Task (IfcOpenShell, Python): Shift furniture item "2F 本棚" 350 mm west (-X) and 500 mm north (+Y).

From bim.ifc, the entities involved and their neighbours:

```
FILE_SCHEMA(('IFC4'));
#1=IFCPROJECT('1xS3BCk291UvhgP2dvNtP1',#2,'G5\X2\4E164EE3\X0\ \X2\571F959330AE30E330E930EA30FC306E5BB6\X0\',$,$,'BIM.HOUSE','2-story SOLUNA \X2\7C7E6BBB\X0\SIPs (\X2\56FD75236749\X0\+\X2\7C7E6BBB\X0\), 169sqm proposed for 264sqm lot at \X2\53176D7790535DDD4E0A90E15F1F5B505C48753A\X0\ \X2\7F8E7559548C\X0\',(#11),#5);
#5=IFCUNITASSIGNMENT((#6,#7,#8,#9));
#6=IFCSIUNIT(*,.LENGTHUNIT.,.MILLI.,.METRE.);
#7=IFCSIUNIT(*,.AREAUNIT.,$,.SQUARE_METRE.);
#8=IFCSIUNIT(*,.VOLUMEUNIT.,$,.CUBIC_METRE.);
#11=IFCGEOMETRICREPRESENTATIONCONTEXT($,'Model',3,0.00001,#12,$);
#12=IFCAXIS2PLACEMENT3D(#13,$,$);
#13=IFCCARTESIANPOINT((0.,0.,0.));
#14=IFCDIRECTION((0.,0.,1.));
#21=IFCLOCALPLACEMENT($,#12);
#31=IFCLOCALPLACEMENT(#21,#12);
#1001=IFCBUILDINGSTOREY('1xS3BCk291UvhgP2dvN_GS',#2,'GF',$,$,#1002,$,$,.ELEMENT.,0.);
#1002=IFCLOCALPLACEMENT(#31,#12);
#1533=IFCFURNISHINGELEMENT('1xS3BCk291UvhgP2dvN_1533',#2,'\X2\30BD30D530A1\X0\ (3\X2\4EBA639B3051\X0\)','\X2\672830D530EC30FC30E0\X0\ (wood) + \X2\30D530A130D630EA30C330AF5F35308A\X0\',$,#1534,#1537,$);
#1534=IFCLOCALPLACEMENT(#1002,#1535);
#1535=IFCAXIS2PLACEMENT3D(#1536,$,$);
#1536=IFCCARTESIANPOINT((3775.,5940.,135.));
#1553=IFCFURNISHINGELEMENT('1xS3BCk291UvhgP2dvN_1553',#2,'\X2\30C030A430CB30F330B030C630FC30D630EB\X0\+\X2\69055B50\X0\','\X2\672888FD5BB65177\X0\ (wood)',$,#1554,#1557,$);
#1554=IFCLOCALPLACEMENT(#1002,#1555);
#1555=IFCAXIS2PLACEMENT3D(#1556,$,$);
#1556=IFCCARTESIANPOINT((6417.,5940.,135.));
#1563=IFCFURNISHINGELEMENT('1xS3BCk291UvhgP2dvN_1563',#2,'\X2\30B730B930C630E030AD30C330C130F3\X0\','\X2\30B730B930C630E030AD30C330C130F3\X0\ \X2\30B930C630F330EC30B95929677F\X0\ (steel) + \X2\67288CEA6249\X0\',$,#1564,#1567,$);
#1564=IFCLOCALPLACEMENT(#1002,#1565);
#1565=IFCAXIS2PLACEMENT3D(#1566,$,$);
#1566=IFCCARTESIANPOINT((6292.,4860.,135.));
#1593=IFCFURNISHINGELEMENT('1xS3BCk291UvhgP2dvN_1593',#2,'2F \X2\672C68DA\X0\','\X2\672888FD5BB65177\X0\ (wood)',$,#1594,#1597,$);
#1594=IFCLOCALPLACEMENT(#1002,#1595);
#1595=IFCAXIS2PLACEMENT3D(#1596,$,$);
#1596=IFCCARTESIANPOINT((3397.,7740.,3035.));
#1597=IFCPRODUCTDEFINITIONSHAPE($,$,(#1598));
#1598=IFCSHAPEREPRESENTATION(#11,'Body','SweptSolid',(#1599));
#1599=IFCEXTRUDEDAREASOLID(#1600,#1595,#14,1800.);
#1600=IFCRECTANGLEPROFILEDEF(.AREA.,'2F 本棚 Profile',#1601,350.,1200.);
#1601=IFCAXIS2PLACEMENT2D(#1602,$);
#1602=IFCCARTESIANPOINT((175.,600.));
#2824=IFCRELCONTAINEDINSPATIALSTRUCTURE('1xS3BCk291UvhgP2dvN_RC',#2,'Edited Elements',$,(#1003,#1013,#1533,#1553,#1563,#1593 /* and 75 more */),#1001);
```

```python
import ifcopenshell
import ifcopenshell.api.geometry
import ifcopenshell.util.placement
import ifcopenshell.util.unit

model = ifcopenshell.open("bim.ifc")
unit_scale = ifcopenshell.util.unit.calculate_unit_scale(model)

item = model.by_guid("1xS3BCk291UvhgP2dvN_1593")
matrix = ifcopenshell.util.placement.get_local_placement(item.ObjectPlacement)
matrix[0, 3] -= 0.35 / unit_scale
matrix[1, 3] += 0.5 / unit_scale
ifcopenshell.api.geometry.edit_object_placement(model, product=item, matrix=matrix, is_si=False)

print(ifcopenshell.util.placement.get_local_placement(item.ObjectPlacement).round(3) + 0.0)

model.write("bim_updated.ifc")
```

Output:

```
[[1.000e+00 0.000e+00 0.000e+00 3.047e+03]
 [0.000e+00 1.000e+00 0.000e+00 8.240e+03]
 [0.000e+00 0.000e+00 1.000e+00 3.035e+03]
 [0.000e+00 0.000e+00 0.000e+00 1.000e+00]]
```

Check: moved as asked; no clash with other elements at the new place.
